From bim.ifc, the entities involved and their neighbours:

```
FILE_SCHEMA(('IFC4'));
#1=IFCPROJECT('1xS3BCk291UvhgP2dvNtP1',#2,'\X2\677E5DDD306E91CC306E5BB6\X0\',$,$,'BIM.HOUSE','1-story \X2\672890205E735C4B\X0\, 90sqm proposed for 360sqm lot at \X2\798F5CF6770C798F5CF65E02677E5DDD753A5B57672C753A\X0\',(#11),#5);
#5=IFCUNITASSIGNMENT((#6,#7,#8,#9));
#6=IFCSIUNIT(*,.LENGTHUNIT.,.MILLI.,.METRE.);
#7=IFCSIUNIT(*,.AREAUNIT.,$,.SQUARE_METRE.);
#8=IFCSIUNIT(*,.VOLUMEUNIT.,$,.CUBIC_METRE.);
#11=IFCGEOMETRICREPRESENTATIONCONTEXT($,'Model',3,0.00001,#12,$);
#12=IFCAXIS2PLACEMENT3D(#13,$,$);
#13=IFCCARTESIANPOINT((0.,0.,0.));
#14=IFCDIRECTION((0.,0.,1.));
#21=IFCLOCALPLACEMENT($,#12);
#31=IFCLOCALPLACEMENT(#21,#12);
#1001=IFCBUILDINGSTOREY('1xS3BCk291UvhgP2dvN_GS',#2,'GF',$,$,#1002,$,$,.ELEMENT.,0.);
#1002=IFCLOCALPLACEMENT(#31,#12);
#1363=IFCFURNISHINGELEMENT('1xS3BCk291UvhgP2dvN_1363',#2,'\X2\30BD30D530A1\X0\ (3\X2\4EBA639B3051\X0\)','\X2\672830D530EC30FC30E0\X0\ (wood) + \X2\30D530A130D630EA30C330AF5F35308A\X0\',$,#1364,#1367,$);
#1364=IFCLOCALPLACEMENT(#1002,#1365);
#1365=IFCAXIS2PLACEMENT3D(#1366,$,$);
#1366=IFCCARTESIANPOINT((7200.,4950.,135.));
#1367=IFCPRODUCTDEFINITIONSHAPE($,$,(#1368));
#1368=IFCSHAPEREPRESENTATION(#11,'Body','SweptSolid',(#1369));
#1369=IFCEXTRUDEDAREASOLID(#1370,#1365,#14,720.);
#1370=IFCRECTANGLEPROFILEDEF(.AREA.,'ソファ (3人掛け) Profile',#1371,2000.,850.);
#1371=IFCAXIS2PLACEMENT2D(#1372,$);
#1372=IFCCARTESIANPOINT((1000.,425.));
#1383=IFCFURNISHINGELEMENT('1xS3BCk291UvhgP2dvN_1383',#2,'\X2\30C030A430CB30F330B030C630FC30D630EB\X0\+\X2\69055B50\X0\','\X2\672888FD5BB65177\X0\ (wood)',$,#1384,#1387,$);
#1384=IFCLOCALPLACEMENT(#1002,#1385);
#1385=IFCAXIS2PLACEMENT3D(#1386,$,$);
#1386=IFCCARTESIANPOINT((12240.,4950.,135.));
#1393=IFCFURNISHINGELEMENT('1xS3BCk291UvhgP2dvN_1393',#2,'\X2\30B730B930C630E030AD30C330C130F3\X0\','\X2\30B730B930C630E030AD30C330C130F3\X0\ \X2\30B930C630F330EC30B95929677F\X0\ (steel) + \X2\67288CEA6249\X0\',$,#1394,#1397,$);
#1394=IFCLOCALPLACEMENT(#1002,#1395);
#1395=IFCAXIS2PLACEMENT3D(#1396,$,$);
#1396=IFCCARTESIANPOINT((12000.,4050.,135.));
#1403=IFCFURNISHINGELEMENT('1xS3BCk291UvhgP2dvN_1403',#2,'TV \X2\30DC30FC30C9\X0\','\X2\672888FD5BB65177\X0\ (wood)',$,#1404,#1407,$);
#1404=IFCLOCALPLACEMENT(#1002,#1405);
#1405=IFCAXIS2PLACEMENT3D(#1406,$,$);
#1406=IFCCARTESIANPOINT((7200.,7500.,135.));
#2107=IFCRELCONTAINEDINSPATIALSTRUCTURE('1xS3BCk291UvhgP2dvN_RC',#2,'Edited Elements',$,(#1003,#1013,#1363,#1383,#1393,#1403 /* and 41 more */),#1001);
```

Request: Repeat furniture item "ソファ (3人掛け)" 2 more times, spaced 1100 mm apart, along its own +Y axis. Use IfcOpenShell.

```python
import ifcopenshell
import ifcopenshell.api.geometry
import ifcopenshell.api.root
import ifcopenshell.util.element
import ifcopenshell.util.placement

model = ifcopenshell.open("bim.ifc")


def reuse_history(source, copy):
    """copy_class also copies each property set's owner history, people and application; keep the originals."""
    for rel in copy.IsDefinedBy:
        if rel.is_a("IfcRelDefinesByProperties") and (history := rel.RelatingPropertyDefinition.OwnerHistory):
            rel.RelatingPropertyDefinition.OwnerHistory = source.OwnerHistory
            ifcopenshell.util.element.remove_deep2(model, history)


source = model.by_guid("1xS3BCk291UvhgP2dvN_1363")
base = ifcopenshell.util.placement.get_local_placement(source.ObjectPlacement)
step = base[:3, 1] * 1100.0

for i in range(1, 3):
    copy = ifcopenshell.api.root.copy_class(model, product=source)
    copy.Representation = ifcopenshell.util.element.copy_deep(
        model, source.Representation, exclude=["IfcGeometricRepresentationContext", "IfcRepresentationMap"]
    )
    reuse_history(source, copy)
    matrix = base.copy()
    matrix[:3, 3] += i * step
    print("added at", matrix[:3, 3].round(3) + 0.0)
    ifcopenshell.api.geometry.edit_object_placement(model, product=copy, matrix=matrix, is_si=False)

model.write("bim_rev.ifc")
```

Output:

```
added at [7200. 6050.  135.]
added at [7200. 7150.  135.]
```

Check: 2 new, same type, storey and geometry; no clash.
